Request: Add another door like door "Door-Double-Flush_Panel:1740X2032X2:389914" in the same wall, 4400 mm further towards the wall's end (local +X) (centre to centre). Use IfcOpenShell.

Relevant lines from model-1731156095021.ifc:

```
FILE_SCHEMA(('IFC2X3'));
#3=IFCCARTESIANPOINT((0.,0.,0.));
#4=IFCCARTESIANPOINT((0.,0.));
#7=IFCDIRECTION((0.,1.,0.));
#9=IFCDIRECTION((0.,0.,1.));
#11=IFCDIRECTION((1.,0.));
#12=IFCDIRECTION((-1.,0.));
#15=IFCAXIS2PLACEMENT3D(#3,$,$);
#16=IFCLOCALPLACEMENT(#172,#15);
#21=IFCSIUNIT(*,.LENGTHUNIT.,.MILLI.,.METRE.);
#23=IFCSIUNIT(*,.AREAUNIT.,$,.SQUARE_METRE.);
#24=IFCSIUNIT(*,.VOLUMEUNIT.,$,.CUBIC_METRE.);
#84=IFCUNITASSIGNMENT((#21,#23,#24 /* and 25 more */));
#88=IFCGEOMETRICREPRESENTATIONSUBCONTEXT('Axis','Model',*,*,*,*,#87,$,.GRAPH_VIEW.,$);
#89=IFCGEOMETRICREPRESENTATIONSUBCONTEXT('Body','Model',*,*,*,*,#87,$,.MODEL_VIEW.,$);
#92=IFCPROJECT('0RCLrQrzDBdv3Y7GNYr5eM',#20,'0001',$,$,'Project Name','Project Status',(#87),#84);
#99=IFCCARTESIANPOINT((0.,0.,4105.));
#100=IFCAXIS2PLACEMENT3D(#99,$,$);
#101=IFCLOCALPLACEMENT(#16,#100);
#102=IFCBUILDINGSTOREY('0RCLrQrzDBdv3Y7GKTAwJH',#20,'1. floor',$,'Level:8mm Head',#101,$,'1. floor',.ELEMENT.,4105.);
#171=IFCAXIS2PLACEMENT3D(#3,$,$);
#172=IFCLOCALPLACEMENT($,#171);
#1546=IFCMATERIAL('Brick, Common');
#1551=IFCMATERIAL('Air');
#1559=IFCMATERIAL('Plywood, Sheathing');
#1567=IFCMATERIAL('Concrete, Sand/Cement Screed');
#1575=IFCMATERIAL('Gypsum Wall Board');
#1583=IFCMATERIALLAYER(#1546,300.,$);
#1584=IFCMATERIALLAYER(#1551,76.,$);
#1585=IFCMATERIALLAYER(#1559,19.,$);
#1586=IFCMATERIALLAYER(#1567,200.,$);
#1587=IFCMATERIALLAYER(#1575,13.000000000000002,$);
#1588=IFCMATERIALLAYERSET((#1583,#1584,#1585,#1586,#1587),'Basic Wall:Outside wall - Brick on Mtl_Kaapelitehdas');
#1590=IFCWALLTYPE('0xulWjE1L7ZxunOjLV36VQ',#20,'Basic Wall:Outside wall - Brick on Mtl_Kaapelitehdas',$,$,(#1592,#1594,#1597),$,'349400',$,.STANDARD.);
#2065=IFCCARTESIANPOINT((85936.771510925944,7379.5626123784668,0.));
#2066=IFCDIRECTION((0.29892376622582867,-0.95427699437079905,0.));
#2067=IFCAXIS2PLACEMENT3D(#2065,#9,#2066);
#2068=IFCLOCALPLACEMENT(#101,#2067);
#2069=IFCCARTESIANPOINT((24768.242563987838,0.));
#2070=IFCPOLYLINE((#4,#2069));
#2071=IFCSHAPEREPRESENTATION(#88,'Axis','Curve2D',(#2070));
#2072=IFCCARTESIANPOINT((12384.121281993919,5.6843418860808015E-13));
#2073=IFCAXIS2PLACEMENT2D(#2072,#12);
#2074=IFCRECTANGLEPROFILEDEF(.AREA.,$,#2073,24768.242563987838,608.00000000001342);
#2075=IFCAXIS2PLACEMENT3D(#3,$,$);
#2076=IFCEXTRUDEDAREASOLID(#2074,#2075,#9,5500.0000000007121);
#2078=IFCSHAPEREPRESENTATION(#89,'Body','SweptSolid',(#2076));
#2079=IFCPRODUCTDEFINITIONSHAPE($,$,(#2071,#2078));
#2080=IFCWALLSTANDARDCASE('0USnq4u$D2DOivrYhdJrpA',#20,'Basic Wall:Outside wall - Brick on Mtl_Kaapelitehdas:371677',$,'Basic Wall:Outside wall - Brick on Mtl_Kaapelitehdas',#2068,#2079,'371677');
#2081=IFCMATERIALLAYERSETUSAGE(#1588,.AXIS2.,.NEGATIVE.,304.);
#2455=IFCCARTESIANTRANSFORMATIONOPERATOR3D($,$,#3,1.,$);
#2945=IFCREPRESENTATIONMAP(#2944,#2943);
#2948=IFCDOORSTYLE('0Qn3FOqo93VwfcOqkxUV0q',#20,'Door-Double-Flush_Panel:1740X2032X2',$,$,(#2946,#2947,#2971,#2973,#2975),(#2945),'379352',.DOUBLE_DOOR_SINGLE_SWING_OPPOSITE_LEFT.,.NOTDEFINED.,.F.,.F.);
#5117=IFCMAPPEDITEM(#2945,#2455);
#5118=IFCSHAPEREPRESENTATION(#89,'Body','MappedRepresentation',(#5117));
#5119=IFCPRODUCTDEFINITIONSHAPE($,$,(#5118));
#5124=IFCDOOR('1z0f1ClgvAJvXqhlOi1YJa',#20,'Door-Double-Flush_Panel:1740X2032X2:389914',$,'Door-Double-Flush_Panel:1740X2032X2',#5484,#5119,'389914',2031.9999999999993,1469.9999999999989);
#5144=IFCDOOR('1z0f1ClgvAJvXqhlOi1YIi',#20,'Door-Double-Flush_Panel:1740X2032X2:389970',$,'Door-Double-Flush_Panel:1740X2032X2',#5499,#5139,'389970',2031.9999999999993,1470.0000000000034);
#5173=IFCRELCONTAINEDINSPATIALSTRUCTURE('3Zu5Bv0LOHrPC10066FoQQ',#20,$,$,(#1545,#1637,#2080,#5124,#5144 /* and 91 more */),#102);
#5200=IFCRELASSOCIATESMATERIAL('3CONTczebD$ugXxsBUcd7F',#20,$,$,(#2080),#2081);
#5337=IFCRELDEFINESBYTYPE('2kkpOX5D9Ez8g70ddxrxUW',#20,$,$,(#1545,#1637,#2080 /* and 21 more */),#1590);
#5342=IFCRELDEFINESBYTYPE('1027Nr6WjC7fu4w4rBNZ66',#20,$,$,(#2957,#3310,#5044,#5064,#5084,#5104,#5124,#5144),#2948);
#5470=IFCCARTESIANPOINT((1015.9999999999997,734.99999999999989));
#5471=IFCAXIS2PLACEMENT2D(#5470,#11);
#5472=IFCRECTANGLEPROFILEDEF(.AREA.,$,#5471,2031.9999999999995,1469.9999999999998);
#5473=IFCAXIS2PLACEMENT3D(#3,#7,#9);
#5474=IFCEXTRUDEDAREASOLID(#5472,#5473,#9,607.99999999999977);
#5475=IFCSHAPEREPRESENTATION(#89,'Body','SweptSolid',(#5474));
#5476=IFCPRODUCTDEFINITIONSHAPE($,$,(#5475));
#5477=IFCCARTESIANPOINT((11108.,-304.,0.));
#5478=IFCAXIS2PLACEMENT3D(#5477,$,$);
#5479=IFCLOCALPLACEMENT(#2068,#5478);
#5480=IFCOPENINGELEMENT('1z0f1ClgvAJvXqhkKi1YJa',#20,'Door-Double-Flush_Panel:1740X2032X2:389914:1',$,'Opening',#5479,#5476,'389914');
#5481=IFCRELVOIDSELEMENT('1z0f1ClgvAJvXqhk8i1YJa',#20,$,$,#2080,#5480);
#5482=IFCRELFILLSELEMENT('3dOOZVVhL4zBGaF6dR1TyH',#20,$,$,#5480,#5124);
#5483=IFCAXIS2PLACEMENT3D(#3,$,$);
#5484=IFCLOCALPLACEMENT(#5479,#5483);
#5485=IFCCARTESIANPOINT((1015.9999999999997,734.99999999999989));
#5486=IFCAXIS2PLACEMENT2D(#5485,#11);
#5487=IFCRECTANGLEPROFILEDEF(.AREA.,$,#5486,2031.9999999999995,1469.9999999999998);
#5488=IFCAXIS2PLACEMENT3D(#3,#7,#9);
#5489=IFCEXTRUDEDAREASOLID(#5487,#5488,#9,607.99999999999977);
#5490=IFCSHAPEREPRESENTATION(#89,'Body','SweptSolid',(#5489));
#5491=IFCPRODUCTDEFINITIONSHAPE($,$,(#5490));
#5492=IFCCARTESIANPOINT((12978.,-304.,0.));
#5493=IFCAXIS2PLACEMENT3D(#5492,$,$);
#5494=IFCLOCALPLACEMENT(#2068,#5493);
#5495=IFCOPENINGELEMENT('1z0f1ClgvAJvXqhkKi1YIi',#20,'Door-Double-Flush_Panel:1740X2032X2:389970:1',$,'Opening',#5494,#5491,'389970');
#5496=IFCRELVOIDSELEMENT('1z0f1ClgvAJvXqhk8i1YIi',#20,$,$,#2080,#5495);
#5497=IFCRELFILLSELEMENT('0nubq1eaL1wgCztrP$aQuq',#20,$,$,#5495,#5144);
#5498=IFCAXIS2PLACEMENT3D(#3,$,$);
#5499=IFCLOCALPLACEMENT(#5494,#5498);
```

```python
import ifcopenshell
import ifcopenshell.api.feature
import ifcopenshell.api.geometry
import ifcopenshell.api.root
import ifcopenshell.geom
import ifcopenshell.util.element
import ifcopenshell.util.placement
import ifcopenshell.util.shape
import ifcopenshell.util.unit

model = ifcopenshell.open("model-1731156095021.ifc")
unit_scale = ifcopenshell.util.unit.calculate_unit_scale(model)
settings = ifcopenshell.geom.settings()


def volume(element):
    """Net volume in cubic metres, openings subtracted."""
    shape = ifcopenshell.geom.create_shape(settings, element)
    return ifcopenshell.util.shape.get_volume(shape.geometry)


def reuse_history(source, copy):
    """copy_class also copies each property set's owner history, people and application; keep the originals."""
    for rel in copy.IsDefinedBy:
        if rel.is_a("IfcRelDefinesByProperties") and (history := rel.RelatingPropertyDefinition.OwnerHistory):
            rel.RelatingPropertyDefinition.OwnerHistory = source.OwnerHistory
            ifcopenshell.util.element.remove_deep2(model, history)


door = model.by_guid("1z0f1ClgvAJvXqhlOi1YJa")
opening = door.FillsVoids[0].RelatingOpeningElement
wall = opening.VoidsElements[0].RelatingBuildingElement
before = volume(wall)
shift = ifcopenshell.util.placement.get_local_placement(wall.ObjectPlacement)[:3, 0] * 4.4 / unit_scale

# copy_class copies the void relationship, type, container and properties, but no geometry.
new_opening = ifcopenshell.api.root.copy_class(model, product=opening)
new_opening.Representation = ifcopenshell.util.element.copy_deep(
    model, opening.Representation, exclude=["IfcGeometricRepresentationContext", "IfcRepresentationMap"]
)
new_opening.Name = "Door-Double-Flush_Panel:1740X2032X2"
new_opening.Tag = None
new_door = ifcopenshell.api.root.copy_class(model, product=door)
new_door.Representation = ifcopenshell.util.element.copy_deep(
    model, door.Representation, exclude=["IfcGeometricRepresentationContext", "IfcRepresentationMap"]
)
new_door.Name = "Door-Double-Flush_Panel:1740X2032X2"
new_door.Tag = None
reuse_history(door, new_door)
fills = ifcopenshell.api.feature.add_filling(model, opening=new_opening, element=new_door)
fills.OwnerHistory = new_door.OwnerHistory  # required in IFC2X3

for old, new in ((opening, new_opening), (door, new_door)):
    matrix = ifcopenshell.util.placement.get_local_placement(old.ObjectPlacement)
    matrix[:3, 3] += shift
    ifcopenshell.api.geometry.edit_object_placement(model, product=new, matrix=matrix, is_si=False)

after = volume(wall)

print(f"wall volume {before:.3f} -> {after:.3f} m3")

model.write("model-1731156095021_edited.ifc")
```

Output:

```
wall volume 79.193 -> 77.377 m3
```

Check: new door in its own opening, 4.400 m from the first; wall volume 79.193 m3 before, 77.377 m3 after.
